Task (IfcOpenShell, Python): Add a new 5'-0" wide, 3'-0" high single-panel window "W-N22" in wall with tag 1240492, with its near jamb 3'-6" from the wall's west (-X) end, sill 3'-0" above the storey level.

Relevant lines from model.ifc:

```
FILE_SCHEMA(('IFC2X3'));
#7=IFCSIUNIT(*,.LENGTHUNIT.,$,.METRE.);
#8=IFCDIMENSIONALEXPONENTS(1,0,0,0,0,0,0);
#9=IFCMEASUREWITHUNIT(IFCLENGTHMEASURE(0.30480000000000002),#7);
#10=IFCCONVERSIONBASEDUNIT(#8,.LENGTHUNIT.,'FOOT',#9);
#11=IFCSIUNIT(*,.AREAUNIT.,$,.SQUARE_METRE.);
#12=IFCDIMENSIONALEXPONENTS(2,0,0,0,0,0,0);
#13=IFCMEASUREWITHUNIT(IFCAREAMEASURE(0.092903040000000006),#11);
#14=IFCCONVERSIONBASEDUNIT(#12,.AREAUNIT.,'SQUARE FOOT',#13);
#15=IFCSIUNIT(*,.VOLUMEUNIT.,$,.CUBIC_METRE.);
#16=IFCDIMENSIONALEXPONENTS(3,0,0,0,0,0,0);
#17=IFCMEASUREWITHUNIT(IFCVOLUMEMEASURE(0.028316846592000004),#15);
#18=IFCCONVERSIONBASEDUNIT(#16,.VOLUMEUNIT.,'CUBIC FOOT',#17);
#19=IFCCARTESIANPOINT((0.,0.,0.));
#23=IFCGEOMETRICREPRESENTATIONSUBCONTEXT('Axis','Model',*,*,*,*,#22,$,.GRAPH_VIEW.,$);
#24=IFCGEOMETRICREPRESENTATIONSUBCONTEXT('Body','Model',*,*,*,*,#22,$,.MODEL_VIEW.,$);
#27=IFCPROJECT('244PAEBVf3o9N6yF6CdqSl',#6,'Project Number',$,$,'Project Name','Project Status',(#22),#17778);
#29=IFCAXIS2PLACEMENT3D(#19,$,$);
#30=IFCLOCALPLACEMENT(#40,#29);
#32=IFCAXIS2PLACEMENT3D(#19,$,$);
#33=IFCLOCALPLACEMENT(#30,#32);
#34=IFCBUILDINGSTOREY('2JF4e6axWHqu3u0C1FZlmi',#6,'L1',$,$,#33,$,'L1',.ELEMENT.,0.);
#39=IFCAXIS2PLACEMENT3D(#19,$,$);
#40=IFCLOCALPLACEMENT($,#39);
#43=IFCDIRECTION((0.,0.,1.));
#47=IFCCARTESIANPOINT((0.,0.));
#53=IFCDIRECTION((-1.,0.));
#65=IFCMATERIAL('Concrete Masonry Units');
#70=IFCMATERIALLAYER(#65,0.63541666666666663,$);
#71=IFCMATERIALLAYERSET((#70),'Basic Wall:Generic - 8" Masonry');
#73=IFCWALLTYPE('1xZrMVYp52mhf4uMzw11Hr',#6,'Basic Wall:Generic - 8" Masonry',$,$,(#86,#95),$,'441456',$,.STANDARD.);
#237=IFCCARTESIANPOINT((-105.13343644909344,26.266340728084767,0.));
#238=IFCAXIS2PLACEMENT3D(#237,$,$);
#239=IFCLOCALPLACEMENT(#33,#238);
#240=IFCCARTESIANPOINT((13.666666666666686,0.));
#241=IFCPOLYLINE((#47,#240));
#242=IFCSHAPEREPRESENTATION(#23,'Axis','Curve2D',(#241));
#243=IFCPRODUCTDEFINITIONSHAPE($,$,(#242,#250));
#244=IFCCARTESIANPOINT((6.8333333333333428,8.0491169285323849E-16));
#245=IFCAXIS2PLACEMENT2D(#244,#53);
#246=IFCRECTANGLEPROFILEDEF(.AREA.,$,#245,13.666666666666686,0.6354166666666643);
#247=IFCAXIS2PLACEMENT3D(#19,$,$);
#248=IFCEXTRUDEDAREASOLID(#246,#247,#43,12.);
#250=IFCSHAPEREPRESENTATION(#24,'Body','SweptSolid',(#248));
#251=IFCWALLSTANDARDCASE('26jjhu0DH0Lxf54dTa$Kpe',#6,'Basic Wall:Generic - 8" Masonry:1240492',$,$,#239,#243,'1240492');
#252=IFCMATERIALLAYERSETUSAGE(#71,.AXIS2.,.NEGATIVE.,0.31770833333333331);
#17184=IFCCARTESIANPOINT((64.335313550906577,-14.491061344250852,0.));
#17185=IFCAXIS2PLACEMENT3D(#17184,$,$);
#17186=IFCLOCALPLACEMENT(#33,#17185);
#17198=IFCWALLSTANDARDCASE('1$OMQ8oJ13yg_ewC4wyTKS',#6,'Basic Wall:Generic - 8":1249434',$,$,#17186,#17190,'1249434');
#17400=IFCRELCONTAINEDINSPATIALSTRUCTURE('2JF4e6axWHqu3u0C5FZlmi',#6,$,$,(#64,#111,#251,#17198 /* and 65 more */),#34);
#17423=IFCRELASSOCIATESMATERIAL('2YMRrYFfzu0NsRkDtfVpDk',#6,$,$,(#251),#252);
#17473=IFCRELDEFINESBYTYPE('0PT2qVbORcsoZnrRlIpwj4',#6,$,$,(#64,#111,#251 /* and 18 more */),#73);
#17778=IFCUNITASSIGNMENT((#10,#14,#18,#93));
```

```python
import numpy as np
import ifcopenshell
import ifcopenshell.api.feature
import ifcopenshell.api.geometry
import ifcopenshell.api.root
import ifcopenshell.api.spatial
import ifcopenshell.api.type
import ifcopenshell.geom
import ifcopenshell.util.element
import ifcopenshell.util.placement
import ifcopenshell.util.representation
import ifcopenshell.util.shape
import ifcopenshell.util.unit

model = ifcopenshell.open("model.ifc")
unit_scale = ifcopenshell.util.unit.calculate_unit_scale(model)
settings = ifcopenshell.geom.settings()


def volume(element):
    """Net volume in cubic metres, openings subtracted."""
    shape = ifcopenshell.geom.create_shape(settings, element)
    return ifcopenshell.util.shape.get_volume(shape.geometry)


wall = model.by_guid("26jjhu0DH0Lxf54dTa$Kpe")
storey = ifcopenshell.util.element.get_container(wall, ifc_class="IfcBuildingStorey")
context = ifcopenshell.util.representation.get_context(model, "Model", "Body", "MODEL_VIEW")
before = volume(wall)

width, height, from_end, sill = 1.524, 0.9144, 1.0668, 0.9144  # metres

# The wall runs along its own X axis, and the end named is its -X end.
wall_shape = ifcopenshell.geom.create_shape(settings, wall)
x, y, z = ifcopenshell.util.shape.get_vertices(wall_shape.geometry).T
start = x.min() + from_end
face, thickness = float(y.min()), float(y.max() - y.min())
wall_matrix = ifcopenshell.util.placement.get_local_placement(wall.ObjectPlacement)
level = ifcopenshell.util.placement.get_local_placement(storey.ObjectPlacement)[2, 3]


def in_wall(x, y):
    """Placement at x, y metres in the wall's axes, at sill height."""
    matrix = wall_matrix.copy()
    matrix[:, 3] = wall_matrix @ np.array([x / unit_scale, y / unit_scale, 0.0, 1.0])
    matrix[2, 3] = level + sill / unit_scale
    return matrix


# Opening: a box that overshoots both wall faces by 50 mm.
opening = ifcopenshell.api.root.create_entity(model, ifc_class="IfcOpeningElement")
box = ifcopenshell.api.geometry.add_wall_representation(
    model, context=context, length=width, height=height, thickness=thickness + 0.1
)
ifcopenshell.api.geometry.assign_representation(model, product=opening, representation=box)
ifcopenshell.api.geometry.edit_object_placement(model, product=opening, matrix=in_wall(start, face - 0.05), is_si=False)
ifcopenshell.api.feature.add_feature(model, feature=opening, element=wall)

window = ifcopenshell.api.root.create_entity(model, ifc_class="IfcWindow", name="W-N22")
window.OverallWidth, window.OverallHeight = width / unit_scale, height / unit_scale
body = ifcopenshell.api.geometry.add_window_representation(
    model,
    context=context,
    overall_width=window.OverallWidth,
    overall_height=window.OverallHeight,
    partition_type="SINGLE_PANEL",
)
ifcopenshell.api.geometry.assign_representation(model, product=window, representation=body)
ifcopenshell.api.spatial.assign_container(model, products=[window], relating_structure=storey)
fills = ifcopenshell.api.feature.add_filling(model, opening=opening, element=window)
fills.OwnerHistory = window.OwnerHistory  # required in IFC2X3

# IFC2X3 keeps the operation on the window style.
style = ifcopenshell.api.root.create_entity(model, ifc_class="IfcWindowStyle", name="W-N22")
style.OperationType, style.ConstructionType = "SINGLE_PANEL", "NOTDEFINED"
style.ParameterTakesPrecedence = style.Sizeable = False
ifcopenshell.api.type.assign_type(model, related_objects=[window], relating_type=style)

# Centre the window in the wall's thickness.
ifcopenshell.api.geometry.edit_object_placement(model, product=window, matrix=in_wall(start, face), is_si=False)
window_shape = ifcopenshell.geom.create_shape(settings, window)
depth = ifcopenshell.util.shape.get_vertices(window_shape.geometry)[:, 1]
offset = face + thickness / 2 - (depth.min() + depth.max()) / 2
ifcopenshell.api.geometry.edit_object_placement(model, product=window, matrix=in_wall(start, offset), is_si=False)

after = volume(wall)

print(f"wall volume {before:.3f} -> {after:.3f} m3")

model.write("model-out.ifc")
```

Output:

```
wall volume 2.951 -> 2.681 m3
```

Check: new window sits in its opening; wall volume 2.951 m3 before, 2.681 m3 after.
